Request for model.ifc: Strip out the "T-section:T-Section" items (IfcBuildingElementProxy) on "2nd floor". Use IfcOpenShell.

First a look at what the model holds.

```python
import ifcopenshell
import ifcopenshell.util.element

model = ifcopenshell.open("model.ifc")
print(model.schema)
storey = next(s for s in model.by_type("IfcBuildingStorey") if s.Name == "2nd floor")
proxies = [e for e in ifcopenshell.util.element.get_decomposition(storey) if e.is_a("IfcBuildingElementProxy")]
seen = {}
for e in proxies:
    element_type = ifcopenshell.util.element.get_type(e)
    name = element_type.Name if element_type not in (None, e) else None
    seen[name] = seen.get(name, 0) + 1
for name, count in sorted(seen.items(), key=str):
    print(count, "x", name)
```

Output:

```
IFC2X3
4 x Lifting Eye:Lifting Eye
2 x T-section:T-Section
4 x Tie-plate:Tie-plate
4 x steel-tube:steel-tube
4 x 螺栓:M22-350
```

```python
import ifcopenshell
import ifcopenshell.api.root
import ifcopenshell.util.element

model = ifcopenshell.open("model.ifc")

storey = next(s for s in model.by_type("IfcBuildingStorey") if s.Name == "2nd floor")
proxies = [e for e in ifcopenshell.util.element.get_decomposition(storey) if e.is_a("IfcBuildingElementProxy")]
targets = [e for e in proxies if (t := ifcopenshell.util.element.get_type(e)) not in (None, e) and t.Name == "T-section:T-Section"]

for e in targets:
    ifcopenshell.api.root.remove_product(model, product=e)
print(len(targets), "removed")

model.write("model-out.ifc")
```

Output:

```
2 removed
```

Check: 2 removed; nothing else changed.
